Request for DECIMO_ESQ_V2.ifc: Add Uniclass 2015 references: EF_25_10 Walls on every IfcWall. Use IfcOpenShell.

First a look at what the model holds.

```python
import ifcopenshell

model = ifcopenshell.open("DECIMO_ESQ_V2.ifc")
print(model.schema)
print("classifications:", [c.Name for c in model.by_type("IfcClassification")])
for ifc_class in ("IfcDoor", "IfcRoof", "IfcStair", "IfcWall", "IfcWindow"):
    print(ifc_class, len(model.by_type(ifc_class)))
```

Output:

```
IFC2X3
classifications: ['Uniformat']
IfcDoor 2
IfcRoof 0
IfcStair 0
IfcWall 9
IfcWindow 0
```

```python
import ifcopenshell
import ifcopenshell.api.classification

model = ifcopenshell.open("DECIMO_ESQ_V2.ifc")

# IFC2X3 requires Source and Edition and has no link from the project to the system.
system = model.create_entity("IfcClassification", Source="NBS", Edition="2015", Name="Uniclass 2015")

codes = {
    "IfcWall": ("EF_25_10", "Walls"),
}
for ifc_class, (code, name) in codes.items():
    products = model.by_type(ifc_class)
    ifcopenshell.api.classification.add_reference(
        model, products=products, classification=system, identification=code, name=name
    )
    print(code, len(products))

model.write("DECIMO_ESQ_V2_rev.ifc")
```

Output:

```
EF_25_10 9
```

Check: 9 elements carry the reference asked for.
